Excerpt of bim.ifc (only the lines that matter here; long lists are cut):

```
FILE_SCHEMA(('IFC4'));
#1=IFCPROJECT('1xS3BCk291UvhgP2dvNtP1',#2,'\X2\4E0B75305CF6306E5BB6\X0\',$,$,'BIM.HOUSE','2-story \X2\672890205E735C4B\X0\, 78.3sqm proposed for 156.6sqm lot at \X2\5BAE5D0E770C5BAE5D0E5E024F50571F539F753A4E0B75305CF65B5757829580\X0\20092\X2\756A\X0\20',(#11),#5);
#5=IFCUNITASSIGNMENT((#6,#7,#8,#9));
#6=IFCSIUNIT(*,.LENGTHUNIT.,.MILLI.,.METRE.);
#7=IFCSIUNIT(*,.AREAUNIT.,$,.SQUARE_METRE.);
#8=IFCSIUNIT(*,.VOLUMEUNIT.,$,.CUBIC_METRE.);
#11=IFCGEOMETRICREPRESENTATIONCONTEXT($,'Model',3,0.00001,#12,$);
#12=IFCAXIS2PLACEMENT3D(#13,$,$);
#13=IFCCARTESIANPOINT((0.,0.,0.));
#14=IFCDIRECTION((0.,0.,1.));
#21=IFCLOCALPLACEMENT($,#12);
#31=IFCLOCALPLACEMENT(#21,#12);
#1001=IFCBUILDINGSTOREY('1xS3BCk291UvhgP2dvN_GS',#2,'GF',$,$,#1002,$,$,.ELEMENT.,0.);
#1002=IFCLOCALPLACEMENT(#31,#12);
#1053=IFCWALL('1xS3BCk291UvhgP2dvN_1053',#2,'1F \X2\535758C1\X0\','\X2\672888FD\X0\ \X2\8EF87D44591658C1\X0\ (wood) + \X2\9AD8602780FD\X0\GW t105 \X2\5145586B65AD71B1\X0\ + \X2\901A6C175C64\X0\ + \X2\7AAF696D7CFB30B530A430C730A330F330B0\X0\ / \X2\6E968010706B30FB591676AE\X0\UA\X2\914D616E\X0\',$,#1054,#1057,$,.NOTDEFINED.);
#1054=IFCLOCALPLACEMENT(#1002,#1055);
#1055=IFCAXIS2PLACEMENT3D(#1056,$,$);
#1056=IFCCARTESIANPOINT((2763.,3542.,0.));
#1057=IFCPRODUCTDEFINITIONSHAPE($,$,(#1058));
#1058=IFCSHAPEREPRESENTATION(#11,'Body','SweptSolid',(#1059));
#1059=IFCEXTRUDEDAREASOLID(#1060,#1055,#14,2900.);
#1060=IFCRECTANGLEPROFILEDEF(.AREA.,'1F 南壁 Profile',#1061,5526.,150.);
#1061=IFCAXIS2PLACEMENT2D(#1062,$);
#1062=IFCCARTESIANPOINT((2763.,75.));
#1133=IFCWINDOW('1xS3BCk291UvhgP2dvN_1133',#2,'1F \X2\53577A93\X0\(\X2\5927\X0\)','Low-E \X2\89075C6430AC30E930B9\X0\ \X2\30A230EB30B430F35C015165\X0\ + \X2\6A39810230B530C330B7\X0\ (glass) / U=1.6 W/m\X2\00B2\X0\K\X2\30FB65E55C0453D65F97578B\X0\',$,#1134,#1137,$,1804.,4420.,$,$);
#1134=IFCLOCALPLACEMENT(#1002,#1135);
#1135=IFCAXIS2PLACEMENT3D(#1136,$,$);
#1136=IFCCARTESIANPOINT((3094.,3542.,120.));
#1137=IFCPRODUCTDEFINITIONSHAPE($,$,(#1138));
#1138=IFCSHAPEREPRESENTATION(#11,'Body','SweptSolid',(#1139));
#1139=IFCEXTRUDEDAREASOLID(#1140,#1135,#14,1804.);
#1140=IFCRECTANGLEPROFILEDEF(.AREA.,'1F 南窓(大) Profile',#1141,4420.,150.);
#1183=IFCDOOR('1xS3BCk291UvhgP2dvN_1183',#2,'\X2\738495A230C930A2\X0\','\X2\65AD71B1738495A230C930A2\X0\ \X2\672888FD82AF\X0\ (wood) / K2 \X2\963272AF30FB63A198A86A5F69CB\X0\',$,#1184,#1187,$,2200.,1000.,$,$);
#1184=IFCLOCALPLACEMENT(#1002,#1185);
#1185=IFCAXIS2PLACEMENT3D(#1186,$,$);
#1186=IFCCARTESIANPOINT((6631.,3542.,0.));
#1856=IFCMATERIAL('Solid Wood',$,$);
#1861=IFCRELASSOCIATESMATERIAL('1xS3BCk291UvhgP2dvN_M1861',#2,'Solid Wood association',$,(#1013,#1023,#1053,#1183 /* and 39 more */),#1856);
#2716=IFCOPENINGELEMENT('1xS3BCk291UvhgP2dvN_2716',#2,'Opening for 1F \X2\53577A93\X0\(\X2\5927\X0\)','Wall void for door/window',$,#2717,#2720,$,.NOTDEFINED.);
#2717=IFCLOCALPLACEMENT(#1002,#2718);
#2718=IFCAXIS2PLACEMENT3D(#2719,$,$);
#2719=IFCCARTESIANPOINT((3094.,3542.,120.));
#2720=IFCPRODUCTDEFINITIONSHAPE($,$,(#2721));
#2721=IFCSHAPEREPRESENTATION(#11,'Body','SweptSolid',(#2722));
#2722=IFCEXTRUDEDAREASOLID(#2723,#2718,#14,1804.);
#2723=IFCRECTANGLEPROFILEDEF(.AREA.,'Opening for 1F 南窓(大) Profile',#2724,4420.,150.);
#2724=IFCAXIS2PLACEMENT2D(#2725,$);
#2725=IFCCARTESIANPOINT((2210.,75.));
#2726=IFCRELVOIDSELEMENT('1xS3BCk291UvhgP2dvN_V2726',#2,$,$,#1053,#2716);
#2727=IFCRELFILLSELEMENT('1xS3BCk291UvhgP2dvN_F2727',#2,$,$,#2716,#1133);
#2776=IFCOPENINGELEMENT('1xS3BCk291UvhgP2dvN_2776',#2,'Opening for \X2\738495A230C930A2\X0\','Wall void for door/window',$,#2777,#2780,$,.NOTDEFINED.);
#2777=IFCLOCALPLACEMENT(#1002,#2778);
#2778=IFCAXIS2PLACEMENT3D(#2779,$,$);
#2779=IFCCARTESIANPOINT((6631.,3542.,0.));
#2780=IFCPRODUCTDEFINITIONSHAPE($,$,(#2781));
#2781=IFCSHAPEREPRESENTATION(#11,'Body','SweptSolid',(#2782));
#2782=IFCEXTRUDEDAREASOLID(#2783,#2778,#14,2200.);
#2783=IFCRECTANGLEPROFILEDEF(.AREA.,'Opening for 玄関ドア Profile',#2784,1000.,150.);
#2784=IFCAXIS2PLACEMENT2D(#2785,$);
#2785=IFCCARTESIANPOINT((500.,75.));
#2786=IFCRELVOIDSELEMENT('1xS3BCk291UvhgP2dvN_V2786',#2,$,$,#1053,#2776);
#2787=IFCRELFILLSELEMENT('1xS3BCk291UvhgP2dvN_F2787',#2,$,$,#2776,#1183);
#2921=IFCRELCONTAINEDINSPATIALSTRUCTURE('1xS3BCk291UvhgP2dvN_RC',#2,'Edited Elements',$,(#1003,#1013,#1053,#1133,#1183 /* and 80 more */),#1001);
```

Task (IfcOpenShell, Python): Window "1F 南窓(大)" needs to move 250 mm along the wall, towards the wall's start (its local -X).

```python
import ifcopenshell
import ifcopenshell.api.geometry
import ifcopenshell.util.placement

model = ifcopenshell.open("bim.ifc")

window = model.by_id(1133)
opening = window.FillsVoids[0].RelatingOpeningElement
wall = opening.VoidsElements[0].RelatingBuildingElement

wall_matrix = ifcopenshell.util.placement.get_local_placement(wall.ObjectPlacement)
shift = wall_matrix[:3, 0] * -250.0
before = ifcopenshell.util.placement.get_local_placement(window.ObjectPlacement)[:3, 3].copy()

# The window is not placed relative to its opening, so move both.
for product in (opening, window):
    matrix = ifcopenshell.util.placement.get_local_placement(product.ObjectPlacement)
    matrix[:3, 3] += shift
    ifcopenshell.api.geometry.edit_object_placement(model, product=product, matrix=matrix, is_si=False)

after = ifcopenshell.util.placement.get_local_placement(window.ObjectPlacement)[:3, 3]
print("window moved by", (after - before).round(3) + 0.0)

model.write("bim_v2.ifc")
```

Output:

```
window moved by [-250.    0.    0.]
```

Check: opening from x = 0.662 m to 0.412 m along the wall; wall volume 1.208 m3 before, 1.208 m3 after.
